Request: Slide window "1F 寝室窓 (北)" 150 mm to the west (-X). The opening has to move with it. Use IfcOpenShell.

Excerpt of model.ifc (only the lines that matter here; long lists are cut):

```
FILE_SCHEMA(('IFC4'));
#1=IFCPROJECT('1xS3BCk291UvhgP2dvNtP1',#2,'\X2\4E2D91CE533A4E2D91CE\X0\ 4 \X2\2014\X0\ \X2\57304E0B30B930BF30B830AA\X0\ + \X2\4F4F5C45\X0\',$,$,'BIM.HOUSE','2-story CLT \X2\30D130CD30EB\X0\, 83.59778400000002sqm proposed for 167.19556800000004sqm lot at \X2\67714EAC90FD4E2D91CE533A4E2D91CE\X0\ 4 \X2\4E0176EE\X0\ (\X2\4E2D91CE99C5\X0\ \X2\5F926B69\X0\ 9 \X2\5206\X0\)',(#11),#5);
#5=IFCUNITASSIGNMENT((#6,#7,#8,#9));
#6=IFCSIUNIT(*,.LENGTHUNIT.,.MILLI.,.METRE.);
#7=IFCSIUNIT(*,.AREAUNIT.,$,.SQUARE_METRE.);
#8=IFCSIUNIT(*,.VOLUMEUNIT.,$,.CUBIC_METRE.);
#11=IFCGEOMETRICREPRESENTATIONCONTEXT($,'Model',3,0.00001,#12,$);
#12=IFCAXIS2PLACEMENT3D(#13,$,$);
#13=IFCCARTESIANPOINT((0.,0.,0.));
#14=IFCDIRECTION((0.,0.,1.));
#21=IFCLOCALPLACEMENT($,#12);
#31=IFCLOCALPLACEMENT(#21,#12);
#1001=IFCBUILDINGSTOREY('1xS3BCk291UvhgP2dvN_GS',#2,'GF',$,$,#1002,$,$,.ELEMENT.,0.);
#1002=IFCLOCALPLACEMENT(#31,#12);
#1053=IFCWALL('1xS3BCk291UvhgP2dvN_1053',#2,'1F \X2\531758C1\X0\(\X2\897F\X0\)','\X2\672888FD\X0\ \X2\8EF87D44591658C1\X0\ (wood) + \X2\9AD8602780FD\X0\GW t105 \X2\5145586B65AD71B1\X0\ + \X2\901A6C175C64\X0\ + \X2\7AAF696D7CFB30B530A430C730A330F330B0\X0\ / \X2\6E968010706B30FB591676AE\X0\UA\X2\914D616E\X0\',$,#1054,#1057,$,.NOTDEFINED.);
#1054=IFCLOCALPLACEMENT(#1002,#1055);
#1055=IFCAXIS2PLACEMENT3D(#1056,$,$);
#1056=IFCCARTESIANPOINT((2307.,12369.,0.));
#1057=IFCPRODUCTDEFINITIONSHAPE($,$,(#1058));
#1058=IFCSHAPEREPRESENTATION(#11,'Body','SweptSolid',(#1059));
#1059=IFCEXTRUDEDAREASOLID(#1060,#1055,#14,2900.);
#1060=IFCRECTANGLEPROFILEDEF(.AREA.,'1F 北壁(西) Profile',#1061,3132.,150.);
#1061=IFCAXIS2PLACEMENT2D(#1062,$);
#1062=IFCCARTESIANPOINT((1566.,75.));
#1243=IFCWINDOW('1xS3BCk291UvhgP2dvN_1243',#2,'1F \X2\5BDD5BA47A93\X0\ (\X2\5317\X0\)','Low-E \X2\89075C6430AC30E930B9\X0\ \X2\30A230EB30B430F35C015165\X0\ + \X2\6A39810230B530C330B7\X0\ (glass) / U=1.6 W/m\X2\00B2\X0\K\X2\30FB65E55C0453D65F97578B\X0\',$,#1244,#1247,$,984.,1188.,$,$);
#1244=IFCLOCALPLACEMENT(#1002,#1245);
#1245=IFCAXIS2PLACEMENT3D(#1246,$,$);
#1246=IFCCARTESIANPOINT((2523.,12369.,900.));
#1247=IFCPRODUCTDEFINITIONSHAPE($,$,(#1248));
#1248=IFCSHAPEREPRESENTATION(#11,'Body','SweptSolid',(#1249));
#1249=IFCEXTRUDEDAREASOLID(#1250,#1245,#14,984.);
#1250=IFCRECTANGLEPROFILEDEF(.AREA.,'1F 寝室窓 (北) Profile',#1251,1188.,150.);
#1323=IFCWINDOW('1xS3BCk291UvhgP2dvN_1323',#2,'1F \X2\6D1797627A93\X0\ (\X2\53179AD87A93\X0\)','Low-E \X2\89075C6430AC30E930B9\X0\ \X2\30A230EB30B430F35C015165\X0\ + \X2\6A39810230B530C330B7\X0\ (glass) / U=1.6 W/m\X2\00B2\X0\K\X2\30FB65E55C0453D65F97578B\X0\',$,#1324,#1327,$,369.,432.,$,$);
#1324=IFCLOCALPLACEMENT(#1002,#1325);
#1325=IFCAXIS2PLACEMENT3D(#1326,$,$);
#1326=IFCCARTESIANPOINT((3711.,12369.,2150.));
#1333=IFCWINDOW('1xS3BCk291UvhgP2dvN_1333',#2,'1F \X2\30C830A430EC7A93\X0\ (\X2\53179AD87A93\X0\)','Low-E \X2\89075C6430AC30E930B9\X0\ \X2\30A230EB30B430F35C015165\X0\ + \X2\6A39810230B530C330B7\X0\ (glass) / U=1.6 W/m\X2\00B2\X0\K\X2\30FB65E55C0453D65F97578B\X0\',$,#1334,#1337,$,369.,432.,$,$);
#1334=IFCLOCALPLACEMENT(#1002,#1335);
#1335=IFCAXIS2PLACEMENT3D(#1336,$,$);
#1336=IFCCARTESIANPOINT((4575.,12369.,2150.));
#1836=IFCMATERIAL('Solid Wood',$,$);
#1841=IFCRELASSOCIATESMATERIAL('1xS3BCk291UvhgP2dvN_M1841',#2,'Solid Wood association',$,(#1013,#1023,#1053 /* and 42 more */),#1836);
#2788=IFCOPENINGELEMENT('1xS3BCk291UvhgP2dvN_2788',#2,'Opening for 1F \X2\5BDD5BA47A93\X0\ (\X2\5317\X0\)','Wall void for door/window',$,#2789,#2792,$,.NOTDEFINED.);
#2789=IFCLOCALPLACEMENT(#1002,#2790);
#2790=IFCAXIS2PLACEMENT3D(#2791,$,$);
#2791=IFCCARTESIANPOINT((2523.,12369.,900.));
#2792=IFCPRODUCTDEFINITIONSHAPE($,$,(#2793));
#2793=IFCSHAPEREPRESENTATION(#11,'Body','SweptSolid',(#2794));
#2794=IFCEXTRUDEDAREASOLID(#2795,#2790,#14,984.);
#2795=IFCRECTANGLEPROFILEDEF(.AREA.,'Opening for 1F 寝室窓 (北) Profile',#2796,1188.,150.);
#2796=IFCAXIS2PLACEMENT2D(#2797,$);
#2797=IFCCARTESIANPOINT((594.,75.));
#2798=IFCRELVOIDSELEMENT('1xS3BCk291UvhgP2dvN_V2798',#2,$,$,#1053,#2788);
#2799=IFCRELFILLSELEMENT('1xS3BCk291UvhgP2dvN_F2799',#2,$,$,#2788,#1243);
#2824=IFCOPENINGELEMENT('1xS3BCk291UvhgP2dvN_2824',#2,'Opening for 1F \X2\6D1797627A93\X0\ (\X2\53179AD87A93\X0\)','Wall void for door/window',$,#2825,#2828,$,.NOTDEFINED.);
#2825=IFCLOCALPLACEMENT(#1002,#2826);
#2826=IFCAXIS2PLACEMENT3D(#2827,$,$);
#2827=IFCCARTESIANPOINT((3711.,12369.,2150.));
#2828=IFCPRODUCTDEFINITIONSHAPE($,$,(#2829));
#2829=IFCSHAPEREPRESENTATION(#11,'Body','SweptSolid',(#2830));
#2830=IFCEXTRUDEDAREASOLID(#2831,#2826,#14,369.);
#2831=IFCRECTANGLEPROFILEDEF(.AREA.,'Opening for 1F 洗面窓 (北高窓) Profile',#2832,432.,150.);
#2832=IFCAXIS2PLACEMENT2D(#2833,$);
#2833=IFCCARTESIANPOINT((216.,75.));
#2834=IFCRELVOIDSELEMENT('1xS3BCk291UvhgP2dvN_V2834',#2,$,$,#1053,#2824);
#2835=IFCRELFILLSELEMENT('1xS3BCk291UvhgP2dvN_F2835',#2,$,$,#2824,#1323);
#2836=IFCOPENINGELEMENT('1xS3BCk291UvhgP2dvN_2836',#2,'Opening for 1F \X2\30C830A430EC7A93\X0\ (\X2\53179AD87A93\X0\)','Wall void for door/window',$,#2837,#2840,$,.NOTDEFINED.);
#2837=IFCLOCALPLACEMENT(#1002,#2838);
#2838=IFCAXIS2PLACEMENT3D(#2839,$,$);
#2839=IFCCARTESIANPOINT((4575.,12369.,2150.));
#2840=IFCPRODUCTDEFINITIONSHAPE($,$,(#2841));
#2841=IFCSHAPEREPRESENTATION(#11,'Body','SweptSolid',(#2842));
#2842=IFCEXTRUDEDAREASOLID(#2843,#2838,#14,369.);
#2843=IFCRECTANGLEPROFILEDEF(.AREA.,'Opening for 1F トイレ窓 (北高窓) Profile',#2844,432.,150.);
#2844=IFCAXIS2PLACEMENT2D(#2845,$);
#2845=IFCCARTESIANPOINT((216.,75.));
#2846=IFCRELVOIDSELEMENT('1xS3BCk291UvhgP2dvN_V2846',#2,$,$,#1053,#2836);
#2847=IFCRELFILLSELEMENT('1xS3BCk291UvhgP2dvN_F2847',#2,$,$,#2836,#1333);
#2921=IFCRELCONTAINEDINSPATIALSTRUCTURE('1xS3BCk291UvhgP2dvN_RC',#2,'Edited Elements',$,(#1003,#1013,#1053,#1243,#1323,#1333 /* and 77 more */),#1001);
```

```python
import ifcopenshell
import ifcopenshell.api.geometry
import ifcopenshell.util.placement
import ifcopenshell.util.unit

model = ifcopenshell.open("model.ifc")
unit_scale = ifcopenshell.util.unit.calculate_unit_scale(model)

window = model.by_guid("1xS3BCk291UvhgP2dvN_1243")
opening = window.FillsVoids[0].RelatingOpeningElement
wall = opening.VoidsElements[0].RelatingBuildingElement

wall_matrix = ifcopenshell.util.placement.get_local_placement(wall.ObjectPlacement)
shift = wall_matrix[:3, 0] * -0.15 / unit_scale
before = ifcopenshell.util.placement.get_local_placement(window.ObjectPlacement)[:3, 3].copy()

# The window is not placed relative to its opening, so move both.
for product in (opening, window):
    matrix = ifcopenshell.util.placement.get_local_placement(product.ObjectPlacement)
    matrix[:3, 3] += shift
    ifcopenshell.api.geometry.edit_object_placement(model, product=product, matrix=matrix, is_si=False)

after = ifcopenshell.util.placement.get_local_placement(window.ObjectPlacement)[:3, 3]
print("window moved by", (after - before).round(3) + 0.0)

model.write("model_v2.ifc")
```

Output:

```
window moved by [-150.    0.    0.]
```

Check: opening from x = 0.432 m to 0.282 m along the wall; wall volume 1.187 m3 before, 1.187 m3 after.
